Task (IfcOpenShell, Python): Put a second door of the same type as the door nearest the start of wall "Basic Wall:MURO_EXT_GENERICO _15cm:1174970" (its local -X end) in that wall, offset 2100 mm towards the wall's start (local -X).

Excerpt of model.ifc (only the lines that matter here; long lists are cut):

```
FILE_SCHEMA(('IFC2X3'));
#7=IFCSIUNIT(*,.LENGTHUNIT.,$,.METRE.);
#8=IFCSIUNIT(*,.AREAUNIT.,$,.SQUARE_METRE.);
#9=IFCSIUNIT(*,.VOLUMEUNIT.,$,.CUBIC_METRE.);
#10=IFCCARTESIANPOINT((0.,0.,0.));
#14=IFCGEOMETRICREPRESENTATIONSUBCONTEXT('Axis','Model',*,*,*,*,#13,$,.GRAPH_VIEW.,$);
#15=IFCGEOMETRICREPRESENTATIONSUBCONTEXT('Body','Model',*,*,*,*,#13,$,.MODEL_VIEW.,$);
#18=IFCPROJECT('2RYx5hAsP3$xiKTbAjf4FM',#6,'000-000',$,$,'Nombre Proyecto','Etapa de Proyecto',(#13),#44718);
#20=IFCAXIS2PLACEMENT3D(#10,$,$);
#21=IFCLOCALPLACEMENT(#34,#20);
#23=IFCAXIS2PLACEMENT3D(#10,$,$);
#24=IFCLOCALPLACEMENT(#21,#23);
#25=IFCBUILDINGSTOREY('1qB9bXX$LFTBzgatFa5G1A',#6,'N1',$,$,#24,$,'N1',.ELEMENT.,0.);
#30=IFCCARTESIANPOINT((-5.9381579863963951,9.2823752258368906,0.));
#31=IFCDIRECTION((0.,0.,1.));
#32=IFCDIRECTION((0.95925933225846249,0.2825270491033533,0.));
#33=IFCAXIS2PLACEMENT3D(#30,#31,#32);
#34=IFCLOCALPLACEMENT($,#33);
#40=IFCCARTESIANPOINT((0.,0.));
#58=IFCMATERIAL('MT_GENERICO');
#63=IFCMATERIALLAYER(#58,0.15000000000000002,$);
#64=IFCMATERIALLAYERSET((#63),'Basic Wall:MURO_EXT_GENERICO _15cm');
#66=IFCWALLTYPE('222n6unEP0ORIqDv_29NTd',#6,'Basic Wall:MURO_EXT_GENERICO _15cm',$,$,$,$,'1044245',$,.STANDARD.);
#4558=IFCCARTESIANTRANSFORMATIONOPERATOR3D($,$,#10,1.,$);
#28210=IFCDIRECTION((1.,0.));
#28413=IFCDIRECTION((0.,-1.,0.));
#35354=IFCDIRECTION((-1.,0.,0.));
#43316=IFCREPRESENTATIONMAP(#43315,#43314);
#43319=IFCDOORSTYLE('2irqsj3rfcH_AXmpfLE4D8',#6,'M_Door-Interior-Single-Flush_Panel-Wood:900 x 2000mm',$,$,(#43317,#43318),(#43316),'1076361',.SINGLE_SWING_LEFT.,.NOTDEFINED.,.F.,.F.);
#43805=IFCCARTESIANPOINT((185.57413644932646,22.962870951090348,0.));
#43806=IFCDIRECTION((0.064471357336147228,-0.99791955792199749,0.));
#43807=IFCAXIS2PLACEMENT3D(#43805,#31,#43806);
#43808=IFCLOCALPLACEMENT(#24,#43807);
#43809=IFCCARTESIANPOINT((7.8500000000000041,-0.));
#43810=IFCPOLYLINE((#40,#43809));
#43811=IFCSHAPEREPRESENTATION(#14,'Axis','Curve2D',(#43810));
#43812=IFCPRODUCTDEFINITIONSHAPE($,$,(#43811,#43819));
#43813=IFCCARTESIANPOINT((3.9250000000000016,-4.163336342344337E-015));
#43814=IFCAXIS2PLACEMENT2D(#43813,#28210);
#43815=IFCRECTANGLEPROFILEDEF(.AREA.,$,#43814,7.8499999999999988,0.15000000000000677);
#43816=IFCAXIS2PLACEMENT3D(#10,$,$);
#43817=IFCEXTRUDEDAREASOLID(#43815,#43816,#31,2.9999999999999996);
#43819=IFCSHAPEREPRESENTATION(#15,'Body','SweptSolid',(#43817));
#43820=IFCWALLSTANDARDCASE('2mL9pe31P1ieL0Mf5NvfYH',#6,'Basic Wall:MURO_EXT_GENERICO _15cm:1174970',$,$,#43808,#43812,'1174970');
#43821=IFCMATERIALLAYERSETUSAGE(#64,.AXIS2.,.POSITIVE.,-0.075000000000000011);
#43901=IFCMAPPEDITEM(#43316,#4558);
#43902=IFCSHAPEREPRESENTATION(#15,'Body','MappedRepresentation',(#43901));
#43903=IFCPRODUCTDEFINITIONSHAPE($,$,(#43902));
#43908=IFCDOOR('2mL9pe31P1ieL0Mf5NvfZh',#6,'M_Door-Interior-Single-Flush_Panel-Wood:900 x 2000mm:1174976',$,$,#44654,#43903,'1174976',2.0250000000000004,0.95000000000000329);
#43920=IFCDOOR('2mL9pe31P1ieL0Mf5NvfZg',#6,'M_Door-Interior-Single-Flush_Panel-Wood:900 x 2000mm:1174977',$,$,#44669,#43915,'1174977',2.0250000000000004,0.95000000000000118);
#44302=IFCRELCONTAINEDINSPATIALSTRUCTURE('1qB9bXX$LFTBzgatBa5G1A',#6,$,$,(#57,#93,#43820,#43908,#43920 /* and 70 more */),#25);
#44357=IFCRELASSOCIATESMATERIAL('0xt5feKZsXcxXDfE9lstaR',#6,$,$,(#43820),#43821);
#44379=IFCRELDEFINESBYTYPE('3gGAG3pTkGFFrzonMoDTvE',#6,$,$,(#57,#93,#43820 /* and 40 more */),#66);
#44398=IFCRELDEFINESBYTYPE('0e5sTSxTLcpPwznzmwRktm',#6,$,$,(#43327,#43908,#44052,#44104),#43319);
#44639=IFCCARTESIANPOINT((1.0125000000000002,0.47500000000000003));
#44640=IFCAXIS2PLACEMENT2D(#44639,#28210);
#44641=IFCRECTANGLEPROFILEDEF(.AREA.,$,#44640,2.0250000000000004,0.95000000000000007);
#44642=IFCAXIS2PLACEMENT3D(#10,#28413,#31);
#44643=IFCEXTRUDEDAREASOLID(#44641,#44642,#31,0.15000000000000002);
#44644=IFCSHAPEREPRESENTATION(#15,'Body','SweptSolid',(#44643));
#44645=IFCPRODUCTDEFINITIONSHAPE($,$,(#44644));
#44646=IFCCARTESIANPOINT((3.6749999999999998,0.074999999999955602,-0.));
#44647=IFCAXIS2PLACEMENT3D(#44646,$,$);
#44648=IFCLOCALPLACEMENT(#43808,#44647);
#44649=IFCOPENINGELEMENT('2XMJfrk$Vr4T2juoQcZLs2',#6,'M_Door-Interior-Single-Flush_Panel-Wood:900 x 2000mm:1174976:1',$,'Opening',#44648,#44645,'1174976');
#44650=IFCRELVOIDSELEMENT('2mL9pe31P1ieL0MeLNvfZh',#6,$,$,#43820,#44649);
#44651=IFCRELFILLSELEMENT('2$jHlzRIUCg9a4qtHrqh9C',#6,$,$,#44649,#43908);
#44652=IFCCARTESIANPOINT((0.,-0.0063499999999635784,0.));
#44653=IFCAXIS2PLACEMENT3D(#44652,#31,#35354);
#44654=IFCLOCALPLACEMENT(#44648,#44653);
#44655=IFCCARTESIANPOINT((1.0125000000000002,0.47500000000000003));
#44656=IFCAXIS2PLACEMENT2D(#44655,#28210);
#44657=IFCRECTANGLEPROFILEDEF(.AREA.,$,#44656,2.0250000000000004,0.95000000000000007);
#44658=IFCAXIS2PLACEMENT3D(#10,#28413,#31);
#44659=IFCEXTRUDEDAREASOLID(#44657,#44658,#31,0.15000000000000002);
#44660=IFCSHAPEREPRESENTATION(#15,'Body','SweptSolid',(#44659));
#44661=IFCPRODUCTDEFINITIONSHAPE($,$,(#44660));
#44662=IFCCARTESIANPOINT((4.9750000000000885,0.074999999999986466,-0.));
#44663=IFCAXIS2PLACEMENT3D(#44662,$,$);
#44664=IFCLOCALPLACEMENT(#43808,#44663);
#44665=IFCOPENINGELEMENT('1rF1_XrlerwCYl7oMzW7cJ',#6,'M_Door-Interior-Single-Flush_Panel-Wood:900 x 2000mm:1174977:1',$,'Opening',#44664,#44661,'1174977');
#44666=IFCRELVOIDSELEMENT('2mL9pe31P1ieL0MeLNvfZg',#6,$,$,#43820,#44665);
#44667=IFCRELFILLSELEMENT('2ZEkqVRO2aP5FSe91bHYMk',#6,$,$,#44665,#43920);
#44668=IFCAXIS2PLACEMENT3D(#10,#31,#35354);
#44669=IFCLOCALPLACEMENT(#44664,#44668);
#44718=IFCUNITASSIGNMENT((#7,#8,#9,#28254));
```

```python
import ifcopenshell
import ifcopenshell.api.feature
import ifcopenshell.api.geometry
import ifcopenshell.api.root
import ifcopenshell.geom
import ifcopenshell.util.element
import ifcopenshell.util.placement
import ifcopenshell.util.shape
import ifcopenshell.util.unit

model = ifcopenshell.open("model.ifc")
unit_scale = ifcopenshell.util.unit.calculate_unit_scale(model)
settings = ifcopenshell.geom.settings()


def volume(element):
    """Net volume in cubic metres, openings subtracted."""
    shape = ifcopenshell.geom.create_shape(settings, element)
    return ifcopenshell.util.shape.get_volume(shape.geometry)


def reuse_history(source, copy):
    """copy_class also copies each property set's owner history, people and application; keep the originals."""
    for rel in copy.IsDefinedBy:
        if rel.is_a("IfcRelDefinesByProperties") and (history := rel.RelatingPropertyDefinition.OwnerHistory):
            rel.RelatingPropertyDefinition.OwnerHistory = source.OwnerHistory
            ifcopenshell.util.element.remove_deep2(model, history)


door = model.by_guid("2mL9pe31P1ieL0Mf5NvfZh")
opening = door.FillsVoids[0].RelatingOpeningElement
wall = opening.VoidsElements[0].RelatingBuildingElement
before = volume(wall)
shift = ifcopenshell.util.placement.get_local_placement(wall.ObjectPlacement)[:3, 0] * -2.1 / unit_scale

# copy_class copies the void relationship, type, container and properties, but no geometry.
new_opening = ifcopenshell.api.root.copy_class(model, product=opening)
new_opening.Representation = ifcopenshell.util.element.copy_deep(
    model, opening.Representation, exclude=["IfcGeometricRepresentationContext", "IfcRepresentationMap"]
)
new_opening.Name = "M_Door-Interior-Single-Flush_Panel-Wood:900 x 2000mm"
new_opening.Tag = None
new_door = ifcopenshell.api.root.copy_class(model, product=door)
new_door.Representation = ifcopenshell.util.element.copy_deep(
    model, door.Representation, exclude=["IfcGeometricRepresentationContext", "IfcRepresentationMap"]
)
new_door.Name = "M_Door-Interior-Single-Flush_Panel-Wood:900 x 2000mm"
new_door.Tag = None
reuse_history(door, new_door)
fills = ifcopenshell.api.feature.add_filling(model, opening=new_opening, element=new_door)
fills.OwnerHistory = new_door.OwnerHistory  # required in IFC2X3

for old, new in ((opening, new_opening), (door, new_door)):
    matrix = ifcopenshell.util.placement.get_local_placement(old.ObjectPlacement)
    matrix[:3, 3] += shift
    ifcopenshell.api.geometry.edit_object_placement(model, product=new, matrix=matrix, is_si=False)

after = volume(wall)

print(f"wall volume {before:.3f} -> {after:.3f} m3")

model.write("model_updated.ifc")
```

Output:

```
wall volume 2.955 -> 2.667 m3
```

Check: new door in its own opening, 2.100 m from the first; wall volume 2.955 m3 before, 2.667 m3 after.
